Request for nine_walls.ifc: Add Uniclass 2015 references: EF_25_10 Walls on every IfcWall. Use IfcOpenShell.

First a look at what the model holds.

```python
import ifcopenshell

model = ifcopenshell.open("nine_walls.ifc")
print(model.schema)
print("classifications:", [c.Name for c in model.by_type("IfcClassification")])
for ifc_class in ("IfcDoor", "IfcRoof", "IfcStair", "IfcWall", "IfcWindow"):
    print(ifc_class, len(model.by_type(ifc_class)))
```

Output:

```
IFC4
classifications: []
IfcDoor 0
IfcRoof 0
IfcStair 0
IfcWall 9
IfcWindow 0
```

```python
import ifcopenshell
import ifcopenshell.api.classification

model = ifcopenshell.open("nine_walls.ifc")

system = ifcopenshell.api.classification.add_classification(model, classification="Uniclass 2015")

codes = {
    "IfcWall": ("EF_25_10", "Walls"),
}
for ifc_class, (code, name) in codes.items():
    products = model.by_type(ifc_class)
    ifcopenshell.api.classification.add_reference(
        model, products=products, classification=system, identification=code, name=name
    )
    print(code, len(products))

model.write("nine_walls-out.ifc")
```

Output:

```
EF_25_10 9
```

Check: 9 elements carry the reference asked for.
